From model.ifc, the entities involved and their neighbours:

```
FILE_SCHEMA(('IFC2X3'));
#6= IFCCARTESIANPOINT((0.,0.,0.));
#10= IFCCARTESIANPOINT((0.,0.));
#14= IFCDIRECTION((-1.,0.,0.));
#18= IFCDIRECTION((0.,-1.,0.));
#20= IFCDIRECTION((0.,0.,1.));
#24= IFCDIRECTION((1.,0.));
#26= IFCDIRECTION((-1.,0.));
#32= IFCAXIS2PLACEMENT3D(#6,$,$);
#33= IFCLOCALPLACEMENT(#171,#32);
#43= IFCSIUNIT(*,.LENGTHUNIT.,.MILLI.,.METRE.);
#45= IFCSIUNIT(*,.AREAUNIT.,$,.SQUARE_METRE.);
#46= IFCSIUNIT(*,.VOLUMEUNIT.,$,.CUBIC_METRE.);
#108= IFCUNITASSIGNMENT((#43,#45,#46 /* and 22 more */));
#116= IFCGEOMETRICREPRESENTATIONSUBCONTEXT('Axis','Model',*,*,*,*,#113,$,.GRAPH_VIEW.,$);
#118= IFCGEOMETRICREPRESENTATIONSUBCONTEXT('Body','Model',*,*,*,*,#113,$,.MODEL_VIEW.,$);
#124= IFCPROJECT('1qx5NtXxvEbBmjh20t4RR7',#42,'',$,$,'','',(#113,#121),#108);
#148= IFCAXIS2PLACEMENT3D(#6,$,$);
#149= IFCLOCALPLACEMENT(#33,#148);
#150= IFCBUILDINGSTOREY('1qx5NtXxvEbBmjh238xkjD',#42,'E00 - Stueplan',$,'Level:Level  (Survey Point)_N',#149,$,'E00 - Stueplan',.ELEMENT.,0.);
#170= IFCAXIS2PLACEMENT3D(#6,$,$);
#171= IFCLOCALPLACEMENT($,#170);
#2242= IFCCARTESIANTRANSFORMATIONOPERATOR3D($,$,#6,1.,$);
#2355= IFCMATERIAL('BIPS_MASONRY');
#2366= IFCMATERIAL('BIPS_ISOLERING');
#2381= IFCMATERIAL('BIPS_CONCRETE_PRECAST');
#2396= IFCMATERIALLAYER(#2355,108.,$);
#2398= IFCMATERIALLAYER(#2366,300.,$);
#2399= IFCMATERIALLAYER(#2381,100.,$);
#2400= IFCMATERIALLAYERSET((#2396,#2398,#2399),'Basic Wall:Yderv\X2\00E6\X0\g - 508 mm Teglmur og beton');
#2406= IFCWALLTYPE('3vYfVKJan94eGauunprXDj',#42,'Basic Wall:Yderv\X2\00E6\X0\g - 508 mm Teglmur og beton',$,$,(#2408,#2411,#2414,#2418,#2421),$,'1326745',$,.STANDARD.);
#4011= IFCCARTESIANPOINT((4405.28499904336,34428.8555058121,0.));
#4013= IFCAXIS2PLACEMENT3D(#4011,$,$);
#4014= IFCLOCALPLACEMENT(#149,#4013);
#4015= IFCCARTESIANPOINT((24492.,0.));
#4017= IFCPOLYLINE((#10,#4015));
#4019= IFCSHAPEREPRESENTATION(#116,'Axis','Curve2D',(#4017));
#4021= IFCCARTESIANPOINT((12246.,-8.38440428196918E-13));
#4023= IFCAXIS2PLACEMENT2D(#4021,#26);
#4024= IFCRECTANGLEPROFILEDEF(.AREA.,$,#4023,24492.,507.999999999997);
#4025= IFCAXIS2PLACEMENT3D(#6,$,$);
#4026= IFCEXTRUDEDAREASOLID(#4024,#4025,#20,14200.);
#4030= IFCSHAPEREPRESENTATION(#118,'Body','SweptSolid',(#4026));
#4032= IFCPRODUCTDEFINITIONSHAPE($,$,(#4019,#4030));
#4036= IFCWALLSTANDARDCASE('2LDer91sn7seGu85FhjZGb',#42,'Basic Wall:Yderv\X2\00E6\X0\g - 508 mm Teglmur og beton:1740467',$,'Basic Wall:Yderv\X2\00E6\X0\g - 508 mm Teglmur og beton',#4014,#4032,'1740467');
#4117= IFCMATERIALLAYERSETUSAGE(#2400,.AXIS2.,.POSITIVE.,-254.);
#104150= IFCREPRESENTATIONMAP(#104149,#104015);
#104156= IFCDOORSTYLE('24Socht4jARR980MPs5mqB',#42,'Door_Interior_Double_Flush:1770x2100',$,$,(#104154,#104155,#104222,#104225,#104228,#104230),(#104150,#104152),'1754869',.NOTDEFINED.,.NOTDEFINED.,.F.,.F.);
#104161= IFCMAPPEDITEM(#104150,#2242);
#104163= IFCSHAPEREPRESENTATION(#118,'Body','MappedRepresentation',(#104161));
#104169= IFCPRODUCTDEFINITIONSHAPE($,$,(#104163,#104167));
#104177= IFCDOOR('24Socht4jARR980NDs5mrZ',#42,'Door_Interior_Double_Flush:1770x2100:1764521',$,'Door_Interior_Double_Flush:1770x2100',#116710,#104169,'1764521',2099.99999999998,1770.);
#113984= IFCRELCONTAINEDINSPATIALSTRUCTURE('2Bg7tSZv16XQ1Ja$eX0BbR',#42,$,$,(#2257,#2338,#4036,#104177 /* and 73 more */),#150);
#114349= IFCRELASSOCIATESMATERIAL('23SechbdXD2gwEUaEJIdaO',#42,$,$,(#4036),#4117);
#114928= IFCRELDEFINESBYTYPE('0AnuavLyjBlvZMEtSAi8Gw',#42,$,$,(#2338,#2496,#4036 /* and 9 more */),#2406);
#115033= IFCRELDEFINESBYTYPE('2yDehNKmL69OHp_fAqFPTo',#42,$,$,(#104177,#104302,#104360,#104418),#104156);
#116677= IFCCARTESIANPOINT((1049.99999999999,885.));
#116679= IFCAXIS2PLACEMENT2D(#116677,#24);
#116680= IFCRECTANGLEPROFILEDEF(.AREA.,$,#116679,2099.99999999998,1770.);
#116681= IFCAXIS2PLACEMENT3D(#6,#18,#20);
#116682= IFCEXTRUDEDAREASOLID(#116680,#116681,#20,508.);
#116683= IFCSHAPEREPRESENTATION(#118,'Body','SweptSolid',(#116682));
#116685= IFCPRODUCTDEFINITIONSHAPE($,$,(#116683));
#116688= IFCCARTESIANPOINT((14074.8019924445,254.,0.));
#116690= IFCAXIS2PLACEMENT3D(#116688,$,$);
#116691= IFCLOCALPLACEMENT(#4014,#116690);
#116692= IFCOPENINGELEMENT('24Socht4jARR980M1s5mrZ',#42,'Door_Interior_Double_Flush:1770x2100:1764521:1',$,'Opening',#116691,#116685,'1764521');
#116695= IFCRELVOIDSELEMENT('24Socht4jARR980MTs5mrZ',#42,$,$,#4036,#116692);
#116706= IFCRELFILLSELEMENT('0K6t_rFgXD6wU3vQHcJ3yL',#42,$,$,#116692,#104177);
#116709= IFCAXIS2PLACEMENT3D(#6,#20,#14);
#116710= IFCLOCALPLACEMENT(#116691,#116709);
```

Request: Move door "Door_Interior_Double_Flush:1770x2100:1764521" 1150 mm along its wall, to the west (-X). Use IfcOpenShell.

```python
import ifcopenshell
import ifcopenshell.api.geometry
import ifcopenshell.util.placement
import ifcopenshell.util.unit

model = ifcopenshell.open("model.ifc")
unit_scale = ifcopenshell.util.unit.calculate_unit_scale(model)

door = model.by_guid("24Socht4jARR980NDs5mrZ")
opening = door.FillsVoids[0].RelatingOpeningElement
wall = opening.VoidsElements[0].RelatingBuildingElement

wall_matrix = ifcopenshell.util.placement.get_local_placement(wall.ObjectPlacement)
shift = wall_matrix[:3, 0] * -1.15 / unit_scale
before = ifcopenshell.util.placement.get_local_placement(door.ObjectPlacement)[:3, 3].copy()

# The door is placed relative to its opening, so it follows when the opening moves.
matrix = ifcopenshell.util.placement.get_local_placement(opening.ObjectPlacement)
matrix[:3, 3] += shift
ifcopenshell.api.geometry.edit_object_placement(
    model, product=opening, matrix=matrix, is_si=False, should_transform_children=True
)

after = ifcopenshell.util.placement.get_local_placement(door.ObjectPlacement)[:3, 3]
print("door moved by", (after - before).round(3) + 0.0)

model.write("model_updated.ifc")
```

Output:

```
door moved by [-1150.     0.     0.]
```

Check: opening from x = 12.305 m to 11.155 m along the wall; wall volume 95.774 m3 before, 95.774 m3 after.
